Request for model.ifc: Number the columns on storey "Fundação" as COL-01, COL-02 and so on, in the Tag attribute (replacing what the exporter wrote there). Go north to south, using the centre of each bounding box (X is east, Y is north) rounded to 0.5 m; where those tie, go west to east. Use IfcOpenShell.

First a look at what the model holds.

```python
import ifcopenshell
import ifcopenshell.util.element
import ifcopenshell.util.placement

model = ifcopenshell.open("model.ifc")
print(model.schema)
storey = next(s for s in model.by_type("IfcBuildingStorey") if s.Name == "Fundação")
columns = [e for e in ifcopenshell.util.element.get_decomposition(storey) if e.is_a("IfcColumn")]
for e in sorted(columns, key=lambda e: e.id()):
    origin = ifcopenshell.util.placement.get_local_placement(e.ObjectPlacement)[:3, 3]
    print(e.id(), e.Tag, e.Name, origin.round(2) + 0.0, sep=" | ")
```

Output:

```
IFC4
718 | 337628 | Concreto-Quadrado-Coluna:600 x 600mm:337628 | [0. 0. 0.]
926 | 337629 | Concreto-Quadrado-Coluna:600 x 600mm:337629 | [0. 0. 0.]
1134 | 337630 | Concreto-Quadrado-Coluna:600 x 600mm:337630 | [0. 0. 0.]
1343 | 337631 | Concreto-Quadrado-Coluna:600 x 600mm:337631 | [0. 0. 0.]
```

```python
import ifcopenshell
import ifcopenshell.geom
import ifcopenshell.util.element
import ifcopenshell.util.shape

model = ifcopenshell.open("model.ifc")
settings = ifcopenshell.geom.settings()
settings.set("use-world-coords", True)


def centre(element):
    shape = ifcopenshell.geom.create_shape(settings, element)
    return ifcopenshell.util.shape.get_bbox_centroid(shape.geometry)


storey = next(s for s in model.by_type("IfcBuildingStorey") if s.Name == "Fundação")
columns = [e for e in ifcopenshell.util.element.get_decomposition(storey) if e.is_a("IfcColumn")]

# Insertion points can sit at a corner or the storey origin, so sort by the geometry (in metres).
centres = {e: centre(e) for e in columns}
columns.sort(key=lambda e: (-round(centres[e][1] / 0.5), centres[e][0]))

for i, e in enumerate(columns, start=1):
    number = f"COL-{i:02d}"
    e.Tag = number
    print(e.id(), number)

model.write("model_rev.ifc")
```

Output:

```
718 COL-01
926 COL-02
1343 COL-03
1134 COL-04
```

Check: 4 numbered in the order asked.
